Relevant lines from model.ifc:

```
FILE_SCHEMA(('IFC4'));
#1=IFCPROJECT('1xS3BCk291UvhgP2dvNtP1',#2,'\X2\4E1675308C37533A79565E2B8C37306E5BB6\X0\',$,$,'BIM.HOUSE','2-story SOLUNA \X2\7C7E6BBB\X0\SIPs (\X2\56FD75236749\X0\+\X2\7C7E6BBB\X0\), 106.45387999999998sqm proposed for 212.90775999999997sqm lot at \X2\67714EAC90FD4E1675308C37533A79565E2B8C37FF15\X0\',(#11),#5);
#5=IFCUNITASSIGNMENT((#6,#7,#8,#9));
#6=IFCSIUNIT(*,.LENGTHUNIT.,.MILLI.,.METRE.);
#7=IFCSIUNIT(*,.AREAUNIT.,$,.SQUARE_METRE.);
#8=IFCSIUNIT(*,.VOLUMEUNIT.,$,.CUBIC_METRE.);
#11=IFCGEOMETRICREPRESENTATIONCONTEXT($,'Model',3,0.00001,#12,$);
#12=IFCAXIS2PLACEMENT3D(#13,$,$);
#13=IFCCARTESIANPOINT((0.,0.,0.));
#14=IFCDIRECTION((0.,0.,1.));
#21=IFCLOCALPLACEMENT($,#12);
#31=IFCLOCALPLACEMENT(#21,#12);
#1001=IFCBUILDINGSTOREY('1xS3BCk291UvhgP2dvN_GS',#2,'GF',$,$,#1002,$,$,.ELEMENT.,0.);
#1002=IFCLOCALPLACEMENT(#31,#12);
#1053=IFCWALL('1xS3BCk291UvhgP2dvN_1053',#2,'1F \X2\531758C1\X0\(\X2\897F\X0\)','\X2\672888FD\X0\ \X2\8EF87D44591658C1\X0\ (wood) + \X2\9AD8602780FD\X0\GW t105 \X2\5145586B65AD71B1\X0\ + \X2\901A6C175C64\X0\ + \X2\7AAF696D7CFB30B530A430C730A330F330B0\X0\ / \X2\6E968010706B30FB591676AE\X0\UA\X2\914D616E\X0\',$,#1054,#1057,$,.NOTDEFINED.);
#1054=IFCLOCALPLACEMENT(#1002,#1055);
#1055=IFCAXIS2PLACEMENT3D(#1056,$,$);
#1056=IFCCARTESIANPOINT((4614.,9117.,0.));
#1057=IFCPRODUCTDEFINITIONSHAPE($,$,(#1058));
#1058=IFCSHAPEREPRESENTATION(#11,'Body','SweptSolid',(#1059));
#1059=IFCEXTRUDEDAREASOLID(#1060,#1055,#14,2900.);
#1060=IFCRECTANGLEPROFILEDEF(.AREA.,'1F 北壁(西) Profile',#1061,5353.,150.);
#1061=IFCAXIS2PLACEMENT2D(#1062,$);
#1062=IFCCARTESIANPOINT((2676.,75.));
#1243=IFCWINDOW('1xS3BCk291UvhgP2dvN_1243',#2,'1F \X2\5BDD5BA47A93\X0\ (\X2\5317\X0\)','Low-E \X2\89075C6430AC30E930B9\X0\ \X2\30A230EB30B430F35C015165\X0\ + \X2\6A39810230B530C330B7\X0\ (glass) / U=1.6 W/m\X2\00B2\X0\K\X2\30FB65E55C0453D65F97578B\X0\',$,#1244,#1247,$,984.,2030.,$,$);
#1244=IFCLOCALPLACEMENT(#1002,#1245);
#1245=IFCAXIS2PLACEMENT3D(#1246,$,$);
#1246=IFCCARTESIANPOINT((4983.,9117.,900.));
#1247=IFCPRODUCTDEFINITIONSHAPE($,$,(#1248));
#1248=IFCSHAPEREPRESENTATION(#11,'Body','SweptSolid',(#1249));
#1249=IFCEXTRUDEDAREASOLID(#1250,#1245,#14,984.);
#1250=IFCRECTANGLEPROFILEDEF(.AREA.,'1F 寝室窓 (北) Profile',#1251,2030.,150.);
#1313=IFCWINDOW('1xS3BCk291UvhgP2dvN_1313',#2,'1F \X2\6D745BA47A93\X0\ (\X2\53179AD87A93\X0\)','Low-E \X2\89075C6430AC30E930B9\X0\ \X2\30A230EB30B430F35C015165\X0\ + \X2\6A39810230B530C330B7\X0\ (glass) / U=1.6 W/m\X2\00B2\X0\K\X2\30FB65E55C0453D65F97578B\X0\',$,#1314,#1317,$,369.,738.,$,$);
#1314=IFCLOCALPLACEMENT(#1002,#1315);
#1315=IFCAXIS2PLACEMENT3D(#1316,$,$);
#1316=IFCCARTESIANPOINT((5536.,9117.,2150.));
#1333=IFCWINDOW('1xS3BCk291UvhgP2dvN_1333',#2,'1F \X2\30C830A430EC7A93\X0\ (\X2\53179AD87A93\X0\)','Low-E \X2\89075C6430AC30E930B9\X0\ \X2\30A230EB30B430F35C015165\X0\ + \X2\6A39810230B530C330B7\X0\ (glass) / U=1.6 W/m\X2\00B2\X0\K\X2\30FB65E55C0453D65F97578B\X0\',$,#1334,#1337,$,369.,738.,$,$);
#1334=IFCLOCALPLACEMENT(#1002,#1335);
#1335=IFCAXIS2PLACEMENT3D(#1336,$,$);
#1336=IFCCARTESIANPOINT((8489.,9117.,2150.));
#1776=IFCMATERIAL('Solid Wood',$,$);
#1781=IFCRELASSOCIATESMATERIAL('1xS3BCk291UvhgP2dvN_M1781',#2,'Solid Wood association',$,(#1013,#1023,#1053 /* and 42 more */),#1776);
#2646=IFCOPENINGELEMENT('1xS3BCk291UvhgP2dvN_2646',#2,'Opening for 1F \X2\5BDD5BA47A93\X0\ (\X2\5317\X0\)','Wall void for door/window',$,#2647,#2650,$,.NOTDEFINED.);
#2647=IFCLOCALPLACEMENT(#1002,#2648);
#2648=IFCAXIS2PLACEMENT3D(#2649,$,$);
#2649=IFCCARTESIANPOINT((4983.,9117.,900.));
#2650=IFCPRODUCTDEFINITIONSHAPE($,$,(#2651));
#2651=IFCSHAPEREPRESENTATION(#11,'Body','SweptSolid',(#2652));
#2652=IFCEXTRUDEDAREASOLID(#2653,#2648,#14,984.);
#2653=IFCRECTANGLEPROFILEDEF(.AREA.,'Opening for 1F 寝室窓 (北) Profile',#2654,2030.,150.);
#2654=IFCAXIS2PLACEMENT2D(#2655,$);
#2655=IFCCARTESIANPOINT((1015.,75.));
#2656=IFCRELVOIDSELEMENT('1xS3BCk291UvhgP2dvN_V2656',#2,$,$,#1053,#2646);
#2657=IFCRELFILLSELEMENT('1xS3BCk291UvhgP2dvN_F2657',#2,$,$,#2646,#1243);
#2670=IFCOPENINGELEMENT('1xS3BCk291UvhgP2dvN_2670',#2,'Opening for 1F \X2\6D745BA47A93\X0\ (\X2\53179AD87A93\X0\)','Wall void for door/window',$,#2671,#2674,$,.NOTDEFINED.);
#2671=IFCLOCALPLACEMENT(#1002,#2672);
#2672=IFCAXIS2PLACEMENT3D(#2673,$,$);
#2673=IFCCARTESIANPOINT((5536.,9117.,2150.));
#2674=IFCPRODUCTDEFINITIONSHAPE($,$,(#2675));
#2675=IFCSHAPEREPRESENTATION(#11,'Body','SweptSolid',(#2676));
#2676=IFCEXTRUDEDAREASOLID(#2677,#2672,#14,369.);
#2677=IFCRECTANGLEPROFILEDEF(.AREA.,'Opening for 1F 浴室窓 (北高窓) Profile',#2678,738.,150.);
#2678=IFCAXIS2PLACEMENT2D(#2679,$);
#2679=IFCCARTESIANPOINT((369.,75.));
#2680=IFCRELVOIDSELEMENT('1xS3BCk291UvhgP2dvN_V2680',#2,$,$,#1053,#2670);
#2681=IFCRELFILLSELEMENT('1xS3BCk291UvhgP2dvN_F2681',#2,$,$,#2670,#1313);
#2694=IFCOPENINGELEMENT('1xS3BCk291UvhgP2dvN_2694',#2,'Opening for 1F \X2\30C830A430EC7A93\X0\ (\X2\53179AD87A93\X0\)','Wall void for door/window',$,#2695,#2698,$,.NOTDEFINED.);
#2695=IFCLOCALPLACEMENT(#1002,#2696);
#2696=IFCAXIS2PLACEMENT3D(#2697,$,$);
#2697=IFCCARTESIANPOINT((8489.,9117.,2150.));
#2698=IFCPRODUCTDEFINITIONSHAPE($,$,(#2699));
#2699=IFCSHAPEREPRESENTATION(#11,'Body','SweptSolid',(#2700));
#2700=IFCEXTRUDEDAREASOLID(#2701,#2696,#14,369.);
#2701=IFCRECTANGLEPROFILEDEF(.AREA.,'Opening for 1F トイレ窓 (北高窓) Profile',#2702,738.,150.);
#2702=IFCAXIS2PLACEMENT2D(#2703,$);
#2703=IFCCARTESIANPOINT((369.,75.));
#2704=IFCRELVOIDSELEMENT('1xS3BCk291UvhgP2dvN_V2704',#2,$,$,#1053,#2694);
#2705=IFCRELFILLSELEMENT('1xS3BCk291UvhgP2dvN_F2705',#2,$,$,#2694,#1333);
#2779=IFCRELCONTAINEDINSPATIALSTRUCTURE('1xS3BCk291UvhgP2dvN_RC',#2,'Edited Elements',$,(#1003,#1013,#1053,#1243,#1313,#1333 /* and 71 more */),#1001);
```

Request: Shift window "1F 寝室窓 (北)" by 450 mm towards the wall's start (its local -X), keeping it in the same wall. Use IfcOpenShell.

```python
import ifcopenshell
import ifcopenshell.api.geometry
import ifcopenshell.util.placement

model = ifcopenshell.open("model.ifc")

window = model.by_guid("1xS3BCk291UvhgP2dvN_1243")
opening = window.FillsVoids[0].RelatingOpeningElement
wall = opening.VoidsElements[0].RelatingBuildingElement

wall_matrix = ifcopenshell.util.placement.get_local_placement(wall.ObjectPlacement)
shift = wall_matrix[:3, 0] * -450.0
before = ifcopenshell.util.placement.get_local_placement(window.ObjectPlacement)[:3, 3].copy()

# The window is not placed relative to its opening, so move both.
for product in (opening, window):
    matrix = ifcopenshell.util.placement.get_local_placement(product.ObjectPlacement)
    matrix[:3, 3] += shift
    ifcopenshell.api.geometry.edit_object_placement(model, product=product, matrix=matrix, is_si=False)

after = ifcopenshell.util.placement.get_local_placement(window.ObjectPlacement)[:3, 3]
print("window moved by", (after - before).round(3) + 0.0)

model.write("model_rev.ifc")
```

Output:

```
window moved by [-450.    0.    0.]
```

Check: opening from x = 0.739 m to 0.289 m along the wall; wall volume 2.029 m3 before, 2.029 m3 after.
